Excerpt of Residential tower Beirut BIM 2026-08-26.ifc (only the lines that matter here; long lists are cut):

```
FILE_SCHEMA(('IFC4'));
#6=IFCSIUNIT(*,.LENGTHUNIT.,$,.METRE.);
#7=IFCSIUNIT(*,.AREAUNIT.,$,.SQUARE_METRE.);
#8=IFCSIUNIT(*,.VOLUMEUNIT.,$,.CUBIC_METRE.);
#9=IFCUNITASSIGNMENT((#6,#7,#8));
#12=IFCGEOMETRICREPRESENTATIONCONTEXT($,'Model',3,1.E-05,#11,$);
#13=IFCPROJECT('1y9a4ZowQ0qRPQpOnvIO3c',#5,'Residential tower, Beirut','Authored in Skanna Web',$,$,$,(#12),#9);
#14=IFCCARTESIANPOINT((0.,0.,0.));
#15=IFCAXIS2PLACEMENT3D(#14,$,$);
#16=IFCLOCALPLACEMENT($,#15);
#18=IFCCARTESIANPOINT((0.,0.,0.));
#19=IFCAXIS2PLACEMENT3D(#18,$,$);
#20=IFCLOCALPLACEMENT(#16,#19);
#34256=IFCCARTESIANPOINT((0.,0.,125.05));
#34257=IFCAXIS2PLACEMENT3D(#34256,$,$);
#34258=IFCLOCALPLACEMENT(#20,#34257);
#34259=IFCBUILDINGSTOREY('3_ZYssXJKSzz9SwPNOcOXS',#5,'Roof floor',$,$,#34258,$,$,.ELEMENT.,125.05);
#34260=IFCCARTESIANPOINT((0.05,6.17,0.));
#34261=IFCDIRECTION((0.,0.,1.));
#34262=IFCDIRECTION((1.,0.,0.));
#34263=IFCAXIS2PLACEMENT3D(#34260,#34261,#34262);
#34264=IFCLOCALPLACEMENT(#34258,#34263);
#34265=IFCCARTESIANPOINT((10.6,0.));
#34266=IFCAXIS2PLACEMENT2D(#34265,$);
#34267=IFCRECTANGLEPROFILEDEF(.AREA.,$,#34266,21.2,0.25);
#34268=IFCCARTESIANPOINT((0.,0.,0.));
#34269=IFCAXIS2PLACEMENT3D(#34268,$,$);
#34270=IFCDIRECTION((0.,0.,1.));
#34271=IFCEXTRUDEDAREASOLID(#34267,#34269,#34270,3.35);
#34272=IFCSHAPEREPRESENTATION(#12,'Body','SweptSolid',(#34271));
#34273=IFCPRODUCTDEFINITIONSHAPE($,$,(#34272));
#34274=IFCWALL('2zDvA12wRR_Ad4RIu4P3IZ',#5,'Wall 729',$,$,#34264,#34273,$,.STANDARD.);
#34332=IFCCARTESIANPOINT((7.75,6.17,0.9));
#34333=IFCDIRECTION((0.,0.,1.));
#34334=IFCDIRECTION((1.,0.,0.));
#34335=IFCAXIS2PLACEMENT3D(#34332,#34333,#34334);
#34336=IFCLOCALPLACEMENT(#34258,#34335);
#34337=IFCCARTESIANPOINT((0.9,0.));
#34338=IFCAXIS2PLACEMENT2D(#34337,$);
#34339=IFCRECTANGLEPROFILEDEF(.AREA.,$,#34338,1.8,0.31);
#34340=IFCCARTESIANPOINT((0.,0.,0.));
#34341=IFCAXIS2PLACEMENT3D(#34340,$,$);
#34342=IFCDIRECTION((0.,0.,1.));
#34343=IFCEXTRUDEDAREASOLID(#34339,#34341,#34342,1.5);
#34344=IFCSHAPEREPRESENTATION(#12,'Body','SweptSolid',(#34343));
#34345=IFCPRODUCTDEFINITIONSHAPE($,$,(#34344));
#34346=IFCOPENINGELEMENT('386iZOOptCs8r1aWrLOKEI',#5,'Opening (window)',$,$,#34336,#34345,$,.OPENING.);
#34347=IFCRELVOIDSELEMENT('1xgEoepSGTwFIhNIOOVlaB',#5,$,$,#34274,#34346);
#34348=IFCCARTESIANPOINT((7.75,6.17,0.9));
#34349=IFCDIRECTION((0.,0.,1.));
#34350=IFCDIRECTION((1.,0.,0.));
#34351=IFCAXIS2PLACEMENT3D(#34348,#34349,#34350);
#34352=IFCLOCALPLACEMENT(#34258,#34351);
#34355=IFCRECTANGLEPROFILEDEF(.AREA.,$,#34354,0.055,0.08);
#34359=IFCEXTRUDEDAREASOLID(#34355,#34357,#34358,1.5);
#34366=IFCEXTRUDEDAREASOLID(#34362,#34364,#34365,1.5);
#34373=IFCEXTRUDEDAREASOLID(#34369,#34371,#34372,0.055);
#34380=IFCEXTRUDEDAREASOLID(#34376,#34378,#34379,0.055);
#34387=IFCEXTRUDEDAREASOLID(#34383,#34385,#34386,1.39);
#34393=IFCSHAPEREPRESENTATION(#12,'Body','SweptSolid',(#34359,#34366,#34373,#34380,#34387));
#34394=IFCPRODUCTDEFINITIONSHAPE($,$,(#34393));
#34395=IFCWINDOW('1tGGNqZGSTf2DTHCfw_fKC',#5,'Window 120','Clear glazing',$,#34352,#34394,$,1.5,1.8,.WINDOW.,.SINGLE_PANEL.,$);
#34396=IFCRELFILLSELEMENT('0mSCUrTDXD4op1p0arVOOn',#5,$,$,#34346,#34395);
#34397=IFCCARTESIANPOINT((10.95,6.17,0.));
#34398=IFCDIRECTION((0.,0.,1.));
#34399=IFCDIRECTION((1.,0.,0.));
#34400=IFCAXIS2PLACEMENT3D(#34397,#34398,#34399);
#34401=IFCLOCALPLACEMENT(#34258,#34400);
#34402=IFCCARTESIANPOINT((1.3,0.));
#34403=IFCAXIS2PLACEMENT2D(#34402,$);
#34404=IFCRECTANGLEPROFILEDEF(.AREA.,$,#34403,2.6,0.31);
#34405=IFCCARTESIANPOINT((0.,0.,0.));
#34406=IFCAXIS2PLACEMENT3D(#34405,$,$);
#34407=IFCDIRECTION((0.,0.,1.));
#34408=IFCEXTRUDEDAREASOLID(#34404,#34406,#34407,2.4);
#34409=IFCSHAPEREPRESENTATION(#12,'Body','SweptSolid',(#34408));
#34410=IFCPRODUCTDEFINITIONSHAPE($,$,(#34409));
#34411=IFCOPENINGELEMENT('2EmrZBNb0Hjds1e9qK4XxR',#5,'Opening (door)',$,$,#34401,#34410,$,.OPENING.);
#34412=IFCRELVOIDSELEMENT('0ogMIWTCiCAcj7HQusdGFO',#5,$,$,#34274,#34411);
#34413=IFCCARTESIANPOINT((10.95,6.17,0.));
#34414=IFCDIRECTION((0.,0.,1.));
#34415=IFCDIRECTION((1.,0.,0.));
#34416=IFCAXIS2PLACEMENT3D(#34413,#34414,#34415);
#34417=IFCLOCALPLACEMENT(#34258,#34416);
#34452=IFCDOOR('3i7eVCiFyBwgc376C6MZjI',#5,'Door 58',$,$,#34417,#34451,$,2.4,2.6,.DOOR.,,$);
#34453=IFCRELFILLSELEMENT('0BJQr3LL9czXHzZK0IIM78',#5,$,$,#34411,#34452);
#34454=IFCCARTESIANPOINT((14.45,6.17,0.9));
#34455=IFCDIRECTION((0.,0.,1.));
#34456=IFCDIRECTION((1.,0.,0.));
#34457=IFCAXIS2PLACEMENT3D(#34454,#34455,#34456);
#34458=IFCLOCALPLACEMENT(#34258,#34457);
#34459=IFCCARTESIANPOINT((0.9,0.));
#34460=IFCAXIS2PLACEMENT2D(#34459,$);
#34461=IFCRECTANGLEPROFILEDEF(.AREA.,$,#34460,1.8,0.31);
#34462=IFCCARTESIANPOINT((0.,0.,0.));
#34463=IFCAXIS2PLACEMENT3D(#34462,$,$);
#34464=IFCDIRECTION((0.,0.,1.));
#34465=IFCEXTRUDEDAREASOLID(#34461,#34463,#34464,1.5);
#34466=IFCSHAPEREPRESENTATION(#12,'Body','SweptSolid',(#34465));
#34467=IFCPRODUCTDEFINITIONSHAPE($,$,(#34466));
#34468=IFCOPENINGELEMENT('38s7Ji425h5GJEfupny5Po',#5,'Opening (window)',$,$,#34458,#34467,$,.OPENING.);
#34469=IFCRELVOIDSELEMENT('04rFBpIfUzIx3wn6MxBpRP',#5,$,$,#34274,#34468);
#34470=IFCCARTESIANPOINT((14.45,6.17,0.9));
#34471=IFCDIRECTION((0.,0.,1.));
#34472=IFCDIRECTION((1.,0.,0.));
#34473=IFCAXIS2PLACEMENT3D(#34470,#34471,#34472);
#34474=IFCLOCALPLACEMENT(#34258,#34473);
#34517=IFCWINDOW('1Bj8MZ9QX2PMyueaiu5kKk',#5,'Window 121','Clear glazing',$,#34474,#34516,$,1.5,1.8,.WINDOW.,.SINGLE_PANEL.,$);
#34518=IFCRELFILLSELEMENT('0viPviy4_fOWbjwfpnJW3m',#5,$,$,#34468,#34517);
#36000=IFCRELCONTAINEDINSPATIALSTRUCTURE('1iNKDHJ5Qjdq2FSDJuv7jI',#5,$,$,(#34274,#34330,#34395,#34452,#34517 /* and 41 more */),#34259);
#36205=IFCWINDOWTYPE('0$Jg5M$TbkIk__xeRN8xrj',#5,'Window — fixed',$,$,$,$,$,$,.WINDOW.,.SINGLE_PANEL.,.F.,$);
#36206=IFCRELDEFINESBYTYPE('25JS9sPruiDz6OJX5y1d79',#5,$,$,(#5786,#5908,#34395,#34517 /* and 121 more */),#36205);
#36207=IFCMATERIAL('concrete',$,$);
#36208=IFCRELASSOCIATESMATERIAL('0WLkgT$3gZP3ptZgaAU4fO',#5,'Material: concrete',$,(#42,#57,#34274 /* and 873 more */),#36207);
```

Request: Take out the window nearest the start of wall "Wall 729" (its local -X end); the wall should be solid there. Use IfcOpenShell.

```python
import ifcopenshell
import ifcopenshell.api.feature
import ifcopenshell.api.root
import ifcopenshell.geom
import ifcopenshell.util.shape

model = ifcopenshell.open("Residential tower Beirut BIM 2026-08-26.ifc")
settings = ifcopenshell.geom.settings()


def volume(element):
    """Net volume in cubic metres, openings subtracted."""
    shape = ifcopenshell.geom.create_shape(settings, element)
    return ifcopenshell.util.shape.get_volume(shape.geometry)


window = model.by_guid("1tGGNqZGSTf2DTHCfw_fKC")
opening = window.FillsVoids[0].RelatingOpeningElement
wall = opening.VoidsElements[0].RelatingBuildingElement
before = volume(wall)

ifcopenshell.api.root.remove_product(model, product=window)
ifcopenshell.api.feature.remove_feature(model, feature=opening)

after = volume(wall)

print(f"wall volume {before:.3f} -> {after:.3f} m3")

model.write("Residential tower Beirut BIM 2026-08-26_rev.ifc")
```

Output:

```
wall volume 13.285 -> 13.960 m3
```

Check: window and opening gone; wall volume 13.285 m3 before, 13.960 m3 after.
